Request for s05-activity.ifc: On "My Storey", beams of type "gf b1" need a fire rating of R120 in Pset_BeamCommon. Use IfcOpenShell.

First a look at what the model holds.

```python
import ifcopenshell
import ifcopenshell.util.element

model = ifcopenshell.open("s05-activity.ifc")
print(model.schema)
storey = next(s for s in model.by_type("IfcBuildingStorey") if s.Name == "My Storey")
beams = [e for e in ifcopenshell.util.element.get_decomposition(storey) if e.is_a("IfcBeam")]
seen = {}
for e in beams:
    element_type = ifcopenshell.util.element.get_type(e)
    key = (element_type.Name if element_type != e and element_type else None, ifcopenshell.util.element.get_pset(e, "Pset_BeamCommon", "FireRating"))
    seen[key] = seen.get(key, 0) + 1
for (name, value), count in sorted(seen.items(), key=str):
    print(count, "x", name, "|", value)
```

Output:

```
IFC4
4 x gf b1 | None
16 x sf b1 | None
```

```python
import ifcopenshell
import ifcopenshell.api.pset
import ifcopenshell.util.element

model = ifcopenshell.open("s05-activity.ifc")

storey = next(s for s in model.by_type("IfcBuildingStorey") if s.Name == "My Storey")
beams = [e for e in ifcopenshell.util.element.get_decomposition(storey) if e.is_a("IfcBeam")]

count = 0
for e in beams:
    element_type = ifcopenshell.util.element.get_type(e)
    if element_type in (None, e) or element_type.Name != "gf b1":
        continue
    # add_pset returns the element's existing set when there is one.
    pset = ifcopenshell.api.pset.add_pset(model, product=e, name="Pset_BeamCommon")
    ifcopenshell.api.pset.edit_pset(model, pset=pset, properties={"FireRating": "R120"})
    count += 1

print(count, "beams updated")

model.write("s05-activity-out.ifc")
```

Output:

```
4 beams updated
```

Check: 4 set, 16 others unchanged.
